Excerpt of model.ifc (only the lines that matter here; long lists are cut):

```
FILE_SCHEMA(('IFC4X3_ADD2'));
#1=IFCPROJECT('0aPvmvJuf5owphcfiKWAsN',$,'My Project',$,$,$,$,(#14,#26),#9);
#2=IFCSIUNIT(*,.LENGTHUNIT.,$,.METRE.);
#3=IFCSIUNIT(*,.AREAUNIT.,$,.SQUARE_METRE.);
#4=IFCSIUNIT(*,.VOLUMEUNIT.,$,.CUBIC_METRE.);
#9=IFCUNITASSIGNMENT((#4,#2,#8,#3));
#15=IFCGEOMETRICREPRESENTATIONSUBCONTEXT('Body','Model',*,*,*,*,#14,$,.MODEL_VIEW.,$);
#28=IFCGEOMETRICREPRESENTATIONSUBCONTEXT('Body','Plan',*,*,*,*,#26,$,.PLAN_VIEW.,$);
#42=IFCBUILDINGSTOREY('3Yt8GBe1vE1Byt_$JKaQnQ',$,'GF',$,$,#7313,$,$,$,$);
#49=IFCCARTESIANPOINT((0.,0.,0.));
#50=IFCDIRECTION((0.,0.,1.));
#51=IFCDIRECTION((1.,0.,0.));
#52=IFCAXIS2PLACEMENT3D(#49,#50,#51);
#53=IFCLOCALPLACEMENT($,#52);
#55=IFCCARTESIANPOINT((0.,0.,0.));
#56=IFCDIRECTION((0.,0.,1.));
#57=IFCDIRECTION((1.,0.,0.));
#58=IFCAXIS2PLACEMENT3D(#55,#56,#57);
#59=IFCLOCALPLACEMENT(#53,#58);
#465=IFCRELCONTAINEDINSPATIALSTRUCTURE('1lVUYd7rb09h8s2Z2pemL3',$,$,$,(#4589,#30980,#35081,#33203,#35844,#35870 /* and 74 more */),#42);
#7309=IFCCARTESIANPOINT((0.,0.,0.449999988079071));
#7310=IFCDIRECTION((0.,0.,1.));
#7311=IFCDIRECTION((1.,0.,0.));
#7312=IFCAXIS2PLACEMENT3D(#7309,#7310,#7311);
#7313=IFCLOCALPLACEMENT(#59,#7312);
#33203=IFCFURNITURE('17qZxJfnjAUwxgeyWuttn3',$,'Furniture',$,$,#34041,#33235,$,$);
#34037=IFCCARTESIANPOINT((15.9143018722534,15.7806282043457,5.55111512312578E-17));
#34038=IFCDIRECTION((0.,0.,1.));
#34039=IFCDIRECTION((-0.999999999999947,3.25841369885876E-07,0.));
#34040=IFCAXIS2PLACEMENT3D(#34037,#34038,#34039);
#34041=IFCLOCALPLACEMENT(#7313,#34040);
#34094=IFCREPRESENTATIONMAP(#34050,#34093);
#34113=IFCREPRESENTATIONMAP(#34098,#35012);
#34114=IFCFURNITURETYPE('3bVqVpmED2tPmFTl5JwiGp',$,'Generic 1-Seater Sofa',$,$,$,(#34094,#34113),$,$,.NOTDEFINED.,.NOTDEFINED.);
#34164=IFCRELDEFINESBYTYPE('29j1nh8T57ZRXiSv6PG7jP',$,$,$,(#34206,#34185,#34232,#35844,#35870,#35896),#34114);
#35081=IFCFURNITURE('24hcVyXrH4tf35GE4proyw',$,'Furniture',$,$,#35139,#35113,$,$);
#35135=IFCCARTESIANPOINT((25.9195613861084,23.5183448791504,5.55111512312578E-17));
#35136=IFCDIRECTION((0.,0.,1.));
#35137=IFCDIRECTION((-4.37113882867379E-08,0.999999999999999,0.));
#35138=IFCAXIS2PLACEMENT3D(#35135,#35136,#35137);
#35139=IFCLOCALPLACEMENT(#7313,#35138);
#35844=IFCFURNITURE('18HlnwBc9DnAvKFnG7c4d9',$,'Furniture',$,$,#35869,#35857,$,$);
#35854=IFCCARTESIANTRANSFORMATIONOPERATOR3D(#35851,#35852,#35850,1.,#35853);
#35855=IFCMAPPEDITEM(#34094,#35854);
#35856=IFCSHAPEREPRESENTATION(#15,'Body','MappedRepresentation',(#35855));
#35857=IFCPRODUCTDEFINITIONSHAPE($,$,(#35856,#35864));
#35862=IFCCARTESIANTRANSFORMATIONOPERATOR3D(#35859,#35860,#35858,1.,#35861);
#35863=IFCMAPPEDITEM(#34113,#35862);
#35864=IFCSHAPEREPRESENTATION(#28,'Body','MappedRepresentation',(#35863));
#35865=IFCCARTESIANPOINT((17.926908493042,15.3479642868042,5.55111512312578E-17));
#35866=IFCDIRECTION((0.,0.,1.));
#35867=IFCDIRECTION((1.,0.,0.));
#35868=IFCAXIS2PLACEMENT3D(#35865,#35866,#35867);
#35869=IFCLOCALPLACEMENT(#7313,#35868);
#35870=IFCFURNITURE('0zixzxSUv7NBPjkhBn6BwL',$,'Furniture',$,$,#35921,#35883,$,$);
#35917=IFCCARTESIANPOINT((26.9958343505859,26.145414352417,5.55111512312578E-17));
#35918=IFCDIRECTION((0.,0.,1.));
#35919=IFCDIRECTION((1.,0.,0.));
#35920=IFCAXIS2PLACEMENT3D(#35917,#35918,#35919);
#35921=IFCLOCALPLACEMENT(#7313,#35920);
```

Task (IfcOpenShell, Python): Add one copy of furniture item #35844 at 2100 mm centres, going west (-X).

```python
import numpy as np
import ifcopenshell
import ifcopenshell.api.geometry
import ifcopenshell.api.root
import ifcopenshell.util.element
import ifcopenshell.util.placement

model = ifcopenshell.open("model.ifc")

source = model.by_guid("18HlnwBc9DnAvKFnG7c4d9")
base = ifcopenshell.util.placement.get_local_placement(source.ObjectPlacement)
step = np.array([-1.0, 0.0, 0.0]) * 2.1

for i in range(1, 2):
    copy = ifcopenshell.api.root.copy_class(model, product=source)
    copy.Representation = ifcopenshell.util.element.copy_deep(
        model, source.Representation, exclude=["IfcGeometricRepresentationContext", "IfcRepresentationMap"]
    )
    matrix = base.copy()
    matrix[:3, 3] += i * step
    print("added at", matrix[:3, 3].round(3) + 0.0)
    ifcopenshell.api.geometry.edit_object_placement(model, product=copy, matrix=matrix, is_si=False)

model.write("model_edited.ifc")
```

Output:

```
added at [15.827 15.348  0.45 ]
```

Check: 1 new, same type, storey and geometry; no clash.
